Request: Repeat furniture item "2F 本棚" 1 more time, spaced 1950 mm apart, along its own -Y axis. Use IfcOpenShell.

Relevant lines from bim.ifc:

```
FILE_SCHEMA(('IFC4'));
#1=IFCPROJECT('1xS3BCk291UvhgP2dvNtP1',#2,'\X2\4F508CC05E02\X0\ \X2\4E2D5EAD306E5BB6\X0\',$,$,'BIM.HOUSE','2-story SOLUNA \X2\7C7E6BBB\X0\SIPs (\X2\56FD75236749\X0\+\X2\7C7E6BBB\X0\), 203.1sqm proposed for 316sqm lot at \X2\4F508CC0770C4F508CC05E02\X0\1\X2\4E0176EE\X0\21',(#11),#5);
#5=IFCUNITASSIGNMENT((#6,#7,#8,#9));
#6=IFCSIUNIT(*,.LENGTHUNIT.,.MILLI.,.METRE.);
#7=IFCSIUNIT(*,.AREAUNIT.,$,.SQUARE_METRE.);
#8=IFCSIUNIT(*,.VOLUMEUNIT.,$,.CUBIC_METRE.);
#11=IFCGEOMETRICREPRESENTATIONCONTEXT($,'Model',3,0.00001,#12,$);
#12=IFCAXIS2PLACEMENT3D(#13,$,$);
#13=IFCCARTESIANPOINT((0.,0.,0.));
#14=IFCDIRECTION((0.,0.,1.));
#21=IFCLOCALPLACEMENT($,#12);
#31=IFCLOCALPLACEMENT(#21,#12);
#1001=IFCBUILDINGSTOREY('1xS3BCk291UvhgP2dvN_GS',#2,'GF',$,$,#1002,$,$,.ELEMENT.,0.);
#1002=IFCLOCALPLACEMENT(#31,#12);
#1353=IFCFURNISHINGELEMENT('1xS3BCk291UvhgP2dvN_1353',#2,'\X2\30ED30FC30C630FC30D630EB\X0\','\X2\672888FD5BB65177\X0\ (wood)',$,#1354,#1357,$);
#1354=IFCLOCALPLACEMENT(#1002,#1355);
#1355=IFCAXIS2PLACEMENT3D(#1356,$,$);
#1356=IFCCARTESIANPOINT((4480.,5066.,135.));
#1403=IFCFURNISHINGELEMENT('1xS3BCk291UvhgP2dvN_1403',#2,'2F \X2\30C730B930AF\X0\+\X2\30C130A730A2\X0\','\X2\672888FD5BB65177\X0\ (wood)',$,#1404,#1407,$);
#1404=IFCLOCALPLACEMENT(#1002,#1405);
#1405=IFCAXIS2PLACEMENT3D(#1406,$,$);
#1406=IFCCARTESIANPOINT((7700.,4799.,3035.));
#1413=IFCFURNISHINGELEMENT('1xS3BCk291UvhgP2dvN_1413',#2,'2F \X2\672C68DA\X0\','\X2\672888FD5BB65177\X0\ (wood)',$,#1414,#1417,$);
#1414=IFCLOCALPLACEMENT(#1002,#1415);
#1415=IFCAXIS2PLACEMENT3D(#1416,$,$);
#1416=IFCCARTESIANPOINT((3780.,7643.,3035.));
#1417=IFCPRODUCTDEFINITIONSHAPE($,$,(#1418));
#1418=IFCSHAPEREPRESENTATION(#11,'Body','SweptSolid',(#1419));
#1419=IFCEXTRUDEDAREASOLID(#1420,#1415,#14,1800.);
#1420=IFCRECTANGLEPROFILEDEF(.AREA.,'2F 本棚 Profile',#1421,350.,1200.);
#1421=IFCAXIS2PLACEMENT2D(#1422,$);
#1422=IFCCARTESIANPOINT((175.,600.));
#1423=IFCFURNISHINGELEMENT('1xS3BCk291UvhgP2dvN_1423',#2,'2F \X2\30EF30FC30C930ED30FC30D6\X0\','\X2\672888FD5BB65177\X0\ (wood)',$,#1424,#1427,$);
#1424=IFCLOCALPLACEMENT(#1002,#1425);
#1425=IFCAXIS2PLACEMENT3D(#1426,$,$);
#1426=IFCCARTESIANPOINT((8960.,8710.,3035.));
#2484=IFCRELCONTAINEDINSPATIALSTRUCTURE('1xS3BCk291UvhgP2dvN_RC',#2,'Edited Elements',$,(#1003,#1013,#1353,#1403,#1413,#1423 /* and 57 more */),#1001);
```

```python
import ifcopenshell
import ifcopenshell.api.geometry
import ifcopenshell.api.root
import ifcopenshell.util.element
import ifcopenshell.util.placement

model = ifcopenshell.open("bim.ifc")


def reuse_history(source, copy):
    """copy_class also copies each property set's owner history, people and application; keep the originals."""
    for rel in copy.IsDefinedBy:
        if rel.is_a("IfcRelDefinesByProperties") and (history := rel.RelatingPropertyDefinition.OwnerHistory):
            rel.RelatingPropertyDefinition.OwnerHistory = source.OwnerHistory
            ifcopenshell.util.element.remove_deep2(model, history)


source = model.by_guid("1xS3BCk291UvhgP2dvN_1413")
base = ifcopenshell.util.placement.get_local_placement(source.ObjectPlacement)
step = -base[:3, 1] * 1950.0

for i in range(1, 2):
    copy = ifcopenshell.api.root.copy_class(model, product=source)
    copy.Representation = ifcopenshell.util.element.copy_deep(
        model, source.Representation, exclude=["IfcGeometricRepresentationContext", "IfcRepresentationMap"]
    )
    reuse_history(source, copy)
    matrix = base.copy()
    matrix[:3, 3] += i * step
    print("added at", matrix[:3, 3].round(3) + 0.0)
    ifcopenshell.api.geometry.edit_object_placement(model, product=copy, matrix=matrix, is_si=False)

model.write("bim-out.ifc")
```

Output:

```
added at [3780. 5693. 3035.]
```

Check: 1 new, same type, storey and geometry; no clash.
